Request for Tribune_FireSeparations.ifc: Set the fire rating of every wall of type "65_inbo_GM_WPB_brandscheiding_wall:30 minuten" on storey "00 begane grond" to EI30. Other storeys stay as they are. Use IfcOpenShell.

First a look at what the model holds.

```python
import ifcopenshell
import ifcopenshell.util.element

model = ifcopenshell.open("Tribune_FireSeparations.ifc")
print(model.schema)
storey = next(s for s in model.by_type("IfcBuildingStorey") if s.Name == "00 begane grond")
walls = [e for e in ifcopenshell.util.element.get_decomposition(storey) if e.is_a("IfcWall")]
seen = {}
for e in walls:
    element_type = ifcopenshell.util.element.get_type(e)
    key = (element_type.Name if element_type != e and element_type else None, ifcopenshell.util.element.get_pset(e, "Pset_WallCommon", "FireRating"))
    seen[key] = seen.get(key, 0) + 1
for (name, value), count in sorted(seen.items(), key=str):
    print(count, "x", name, "|", value)
```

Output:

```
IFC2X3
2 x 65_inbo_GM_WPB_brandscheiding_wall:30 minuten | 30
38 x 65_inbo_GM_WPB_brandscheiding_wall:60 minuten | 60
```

```python
import ifcopenshell
import ifcopenshell.api.pset
import ifcopenshell.util.element

model = ifcopenshell.open("Tribune_FireSeparations.ifc")

storey = next(s for s in model.by_type("IfcBuildingStorey") if s.Name == "00 begane grond")
walls = [e for e in ifcopenshell.util.element.get_decomposition(storey) if e.is_a("IfcWall")]

count = 0
for e in walls:
    element_type = ifcopenshell.util.element.get_type(e)
    if element_type in (None, e) or element_type.Name != "65_inbo_GM_WPB_brandscheiding_wall:30 minuten":
        continue
    found = ifcopenshell.util.element.get_pset(e, "Pset_WallCommon", should_inherit=False)
    if found:
        pset = model.by_id(found["id"])
        if len(ifcopenshell.util.element.get_elements_by_pset(pset)) > 1:
            pset = ifcopenshell.api.pset.unshare_pset(model, products=[e], pset=pset)[0]
    else:
        pset = ifcopenshell.api.pset.add_pset(model, product=e, name="Pset_WallCommon")
    ifcopenshell.api.pset.edit_pset(model, pset=pset, properties={"FireRating": "EI30"})
    count += 1

print(count, "walls updated")

model.write("Tribune_FireSeparations_rev.ifc")
```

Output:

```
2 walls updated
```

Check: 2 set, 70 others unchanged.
